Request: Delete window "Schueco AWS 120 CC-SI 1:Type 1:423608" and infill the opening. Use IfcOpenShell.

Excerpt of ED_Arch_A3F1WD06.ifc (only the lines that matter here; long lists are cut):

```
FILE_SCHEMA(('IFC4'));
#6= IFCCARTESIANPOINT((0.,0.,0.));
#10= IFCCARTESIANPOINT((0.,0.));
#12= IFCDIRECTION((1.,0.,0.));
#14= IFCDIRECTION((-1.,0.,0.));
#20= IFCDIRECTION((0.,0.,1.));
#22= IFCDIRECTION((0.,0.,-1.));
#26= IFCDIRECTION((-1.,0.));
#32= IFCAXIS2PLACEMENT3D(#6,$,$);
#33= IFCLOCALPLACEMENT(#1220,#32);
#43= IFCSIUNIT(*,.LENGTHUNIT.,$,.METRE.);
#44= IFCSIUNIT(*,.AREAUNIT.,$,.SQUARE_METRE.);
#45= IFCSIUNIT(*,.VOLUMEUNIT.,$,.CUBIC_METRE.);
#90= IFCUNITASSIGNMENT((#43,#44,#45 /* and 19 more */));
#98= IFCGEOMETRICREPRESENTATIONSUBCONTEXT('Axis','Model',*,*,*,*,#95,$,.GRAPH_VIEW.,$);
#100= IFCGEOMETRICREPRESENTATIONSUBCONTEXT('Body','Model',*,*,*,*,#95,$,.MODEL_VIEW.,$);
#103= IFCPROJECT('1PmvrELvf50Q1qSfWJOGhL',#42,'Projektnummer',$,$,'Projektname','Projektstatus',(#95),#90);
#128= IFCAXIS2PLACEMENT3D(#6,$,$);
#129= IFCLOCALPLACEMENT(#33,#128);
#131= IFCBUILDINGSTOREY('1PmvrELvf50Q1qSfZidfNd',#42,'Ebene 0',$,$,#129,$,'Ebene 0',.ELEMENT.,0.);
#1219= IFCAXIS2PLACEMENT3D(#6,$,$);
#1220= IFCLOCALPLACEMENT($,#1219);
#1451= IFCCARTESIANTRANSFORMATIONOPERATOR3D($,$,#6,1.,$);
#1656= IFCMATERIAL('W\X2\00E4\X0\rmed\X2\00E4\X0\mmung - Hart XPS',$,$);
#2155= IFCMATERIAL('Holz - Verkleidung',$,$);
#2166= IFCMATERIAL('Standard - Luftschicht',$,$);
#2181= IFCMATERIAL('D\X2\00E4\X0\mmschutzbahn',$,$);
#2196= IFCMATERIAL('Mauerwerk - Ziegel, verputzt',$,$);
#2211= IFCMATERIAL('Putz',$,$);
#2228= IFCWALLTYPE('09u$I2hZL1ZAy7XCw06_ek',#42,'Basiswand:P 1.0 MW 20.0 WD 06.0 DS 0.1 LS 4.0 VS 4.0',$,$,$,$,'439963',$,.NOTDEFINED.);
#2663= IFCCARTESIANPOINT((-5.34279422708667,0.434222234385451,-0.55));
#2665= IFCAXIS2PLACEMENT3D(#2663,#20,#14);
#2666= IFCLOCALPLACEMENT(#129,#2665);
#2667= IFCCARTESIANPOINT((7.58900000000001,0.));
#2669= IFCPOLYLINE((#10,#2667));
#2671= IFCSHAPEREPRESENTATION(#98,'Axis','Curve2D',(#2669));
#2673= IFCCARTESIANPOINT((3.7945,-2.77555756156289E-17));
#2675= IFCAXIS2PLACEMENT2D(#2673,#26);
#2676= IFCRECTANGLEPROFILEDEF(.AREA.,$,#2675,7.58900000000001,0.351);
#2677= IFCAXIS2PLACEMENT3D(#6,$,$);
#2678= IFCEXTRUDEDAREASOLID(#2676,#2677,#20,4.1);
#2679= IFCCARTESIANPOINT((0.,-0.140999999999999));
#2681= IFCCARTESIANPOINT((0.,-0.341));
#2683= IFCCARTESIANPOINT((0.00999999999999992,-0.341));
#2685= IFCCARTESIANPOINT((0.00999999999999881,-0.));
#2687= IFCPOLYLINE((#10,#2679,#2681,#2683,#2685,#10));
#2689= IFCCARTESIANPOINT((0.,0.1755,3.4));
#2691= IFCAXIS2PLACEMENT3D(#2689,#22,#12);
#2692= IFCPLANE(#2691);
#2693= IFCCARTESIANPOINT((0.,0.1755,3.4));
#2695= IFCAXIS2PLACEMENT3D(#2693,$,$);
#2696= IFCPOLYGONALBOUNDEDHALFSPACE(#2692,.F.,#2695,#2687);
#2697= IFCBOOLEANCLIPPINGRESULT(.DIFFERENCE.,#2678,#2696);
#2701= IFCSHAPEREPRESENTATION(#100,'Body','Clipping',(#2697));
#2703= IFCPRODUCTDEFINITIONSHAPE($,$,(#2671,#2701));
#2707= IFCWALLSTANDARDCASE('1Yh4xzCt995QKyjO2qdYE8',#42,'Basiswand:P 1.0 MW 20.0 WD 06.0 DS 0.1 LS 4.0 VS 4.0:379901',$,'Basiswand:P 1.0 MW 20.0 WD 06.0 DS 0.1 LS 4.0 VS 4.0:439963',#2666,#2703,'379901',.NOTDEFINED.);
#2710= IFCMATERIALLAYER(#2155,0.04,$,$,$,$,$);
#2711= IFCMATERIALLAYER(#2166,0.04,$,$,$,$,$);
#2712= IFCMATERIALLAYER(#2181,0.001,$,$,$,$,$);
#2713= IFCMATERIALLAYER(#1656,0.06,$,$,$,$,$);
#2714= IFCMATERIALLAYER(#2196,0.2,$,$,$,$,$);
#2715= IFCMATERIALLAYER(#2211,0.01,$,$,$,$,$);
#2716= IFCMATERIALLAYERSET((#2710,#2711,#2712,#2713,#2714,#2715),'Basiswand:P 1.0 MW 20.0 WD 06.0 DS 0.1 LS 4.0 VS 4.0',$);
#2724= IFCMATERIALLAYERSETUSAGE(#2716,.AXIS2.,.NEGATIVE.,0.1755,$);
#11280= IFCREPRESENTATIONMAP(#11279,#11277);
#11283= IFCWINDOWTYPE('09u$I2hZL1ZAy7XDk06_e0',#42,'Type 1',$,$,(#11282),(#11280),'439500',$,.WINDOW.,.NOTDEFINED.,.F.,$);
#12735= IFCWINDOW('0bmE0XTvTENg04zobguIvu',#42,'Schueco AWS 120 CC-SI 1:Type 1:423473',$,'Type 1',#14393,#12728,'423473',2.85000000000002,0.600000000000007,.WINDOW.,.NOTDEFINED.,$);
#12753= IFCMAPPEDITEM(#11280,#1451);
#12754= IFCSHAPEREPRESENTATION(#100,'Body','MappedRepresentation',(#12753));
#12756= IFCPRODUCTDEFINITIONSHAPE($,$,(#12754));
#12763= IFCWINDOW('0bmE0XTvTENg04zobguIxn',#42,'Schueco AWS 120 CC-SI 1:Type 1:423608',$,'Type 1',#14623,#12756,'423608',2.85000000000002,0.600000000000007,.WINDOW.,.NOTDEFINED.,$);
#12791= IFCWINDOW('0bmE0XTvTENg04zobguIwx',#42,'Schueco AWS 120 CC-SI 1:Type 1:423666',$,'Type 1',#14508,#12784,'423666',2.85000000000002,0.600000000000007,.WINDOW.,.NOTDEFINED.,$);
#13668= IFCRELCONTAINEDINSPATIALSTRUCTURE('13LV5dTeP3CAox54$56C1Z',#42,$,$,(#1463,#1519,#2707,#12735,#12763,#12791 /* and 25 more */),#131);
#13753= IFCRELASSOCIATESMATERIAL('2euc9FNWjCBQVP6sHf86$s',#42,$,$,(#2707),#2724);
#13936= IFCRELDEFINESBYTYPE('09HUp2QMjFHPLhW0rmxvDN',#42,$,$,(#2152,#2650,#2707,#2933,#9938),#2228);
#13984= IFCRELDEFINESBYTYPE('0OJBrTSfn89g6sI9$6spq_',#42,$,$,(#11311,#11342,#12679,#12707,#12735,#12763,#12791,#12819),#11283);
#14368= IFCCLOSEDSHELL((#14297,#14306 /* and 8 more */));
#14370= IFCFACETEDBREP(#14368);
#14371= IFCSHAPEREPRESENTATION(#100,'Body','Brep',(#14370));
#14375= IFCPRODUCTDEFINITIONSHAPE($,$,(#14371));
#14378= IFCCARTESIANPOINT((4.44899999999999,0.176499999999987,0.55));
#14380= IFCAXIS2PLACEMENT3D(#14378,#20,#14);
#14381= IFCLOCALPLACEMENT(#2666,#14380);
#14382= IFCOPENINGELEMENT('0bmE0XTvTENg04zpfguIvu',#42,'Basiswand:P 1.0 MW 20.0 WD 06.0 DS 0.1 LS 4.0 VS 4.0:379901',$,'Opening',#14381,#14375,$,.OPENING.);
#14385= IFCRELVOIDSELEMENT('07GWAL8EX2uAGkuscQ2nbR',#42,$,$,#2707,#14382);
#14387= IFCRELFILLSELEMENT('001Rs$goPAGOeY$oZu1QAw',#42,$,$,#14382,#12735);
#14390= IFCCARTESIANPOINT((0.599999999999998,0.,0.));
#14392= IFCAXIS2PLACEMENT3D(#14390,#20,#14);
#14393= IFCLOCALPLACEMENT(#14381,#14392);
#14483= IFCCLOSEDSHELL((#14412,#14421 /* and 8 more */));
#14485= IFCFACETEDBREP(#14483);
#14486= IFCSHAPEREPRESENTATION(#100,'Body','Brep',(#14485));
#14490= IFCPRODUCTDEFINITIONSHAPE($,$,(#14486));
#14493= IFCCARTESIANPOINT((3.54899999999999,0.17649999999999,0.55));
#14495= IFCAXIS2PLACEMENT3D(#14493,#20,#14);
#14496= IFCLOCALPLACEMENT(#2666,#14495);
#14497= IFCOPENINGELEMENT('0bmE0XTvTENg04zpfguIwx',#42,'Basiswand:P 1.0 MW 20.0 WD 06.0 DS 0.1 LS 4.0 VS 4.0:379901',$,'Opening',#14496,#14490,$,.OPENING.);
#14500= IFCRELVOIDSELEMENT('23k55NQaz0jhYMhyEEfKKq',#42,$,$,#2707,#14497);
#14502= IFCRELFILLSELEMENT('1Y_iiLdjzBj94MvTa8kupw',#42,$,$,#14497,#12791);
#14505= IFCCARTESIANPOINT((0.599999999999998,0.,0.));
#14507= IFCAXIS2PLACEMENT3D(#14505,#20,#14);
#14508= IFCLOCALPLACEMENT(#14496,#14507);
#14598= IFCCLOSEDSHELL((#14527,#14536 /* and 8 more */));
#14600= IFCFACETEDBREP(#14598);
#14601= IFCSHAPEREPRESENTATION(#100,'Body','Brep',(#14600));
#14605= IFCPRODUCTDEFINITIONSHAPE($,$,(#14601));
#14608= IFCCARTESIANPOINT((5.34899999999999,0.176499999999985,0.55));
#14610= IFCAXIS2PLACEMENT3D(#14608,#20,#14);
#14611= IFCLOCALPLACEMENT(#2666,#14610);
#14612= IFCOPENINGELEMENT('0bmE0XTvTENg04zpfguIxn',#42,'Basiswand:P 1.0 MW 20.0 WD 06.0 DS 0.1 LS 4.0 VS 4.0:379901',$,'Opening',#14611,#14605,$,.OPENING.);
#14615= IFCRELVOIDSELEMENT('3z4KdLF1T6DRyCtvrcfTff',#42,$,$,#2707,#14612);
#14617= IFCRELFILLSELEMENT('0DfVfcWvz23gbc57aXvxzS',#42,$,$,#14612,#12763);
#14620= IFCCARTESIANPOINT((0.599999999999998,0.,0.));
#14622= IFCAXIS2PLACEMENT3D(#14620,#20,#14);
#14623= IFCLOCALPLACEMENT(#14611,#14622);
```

```python
import ifcopenshell
import ifcopenshell.api.feature
import ifcopenshell.api.root
import ifcopenshell.geom
import ifcopenshell.util.shape

model = ifcopenshell.open("ED_Arch_A3F1WD06.ifc")
settings = ifcopenshell.geom.settings()


def volume(element):
    """Net volume in cubic metres, openings subtracted."""
    shape = ifcopenshell.geom.create_shape(settings, element)
    return ifcopenshell.util.shape.get_volume(shape.geometry)


window = model.by_id(12763)
opening = window.FillsVoids[0].RelatingOpeningElement
wall = opening.VoidsElements[0].RelatingBuildingElement
before = volume(wall)

ifcopenshell.api.root.remove_product(model, product=window)
ifcopenshell.api.feature.remove_feature(model, feature=opening)

after = volume(wall)

print(f"wall volume {before:.3f} -> {after:.3f} m3")

model.write("ED_Arch_A3F1WD06_updated.ifc")
```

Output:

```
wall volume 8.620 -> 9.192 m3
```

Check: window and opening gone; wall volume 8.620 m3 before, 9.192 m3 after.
